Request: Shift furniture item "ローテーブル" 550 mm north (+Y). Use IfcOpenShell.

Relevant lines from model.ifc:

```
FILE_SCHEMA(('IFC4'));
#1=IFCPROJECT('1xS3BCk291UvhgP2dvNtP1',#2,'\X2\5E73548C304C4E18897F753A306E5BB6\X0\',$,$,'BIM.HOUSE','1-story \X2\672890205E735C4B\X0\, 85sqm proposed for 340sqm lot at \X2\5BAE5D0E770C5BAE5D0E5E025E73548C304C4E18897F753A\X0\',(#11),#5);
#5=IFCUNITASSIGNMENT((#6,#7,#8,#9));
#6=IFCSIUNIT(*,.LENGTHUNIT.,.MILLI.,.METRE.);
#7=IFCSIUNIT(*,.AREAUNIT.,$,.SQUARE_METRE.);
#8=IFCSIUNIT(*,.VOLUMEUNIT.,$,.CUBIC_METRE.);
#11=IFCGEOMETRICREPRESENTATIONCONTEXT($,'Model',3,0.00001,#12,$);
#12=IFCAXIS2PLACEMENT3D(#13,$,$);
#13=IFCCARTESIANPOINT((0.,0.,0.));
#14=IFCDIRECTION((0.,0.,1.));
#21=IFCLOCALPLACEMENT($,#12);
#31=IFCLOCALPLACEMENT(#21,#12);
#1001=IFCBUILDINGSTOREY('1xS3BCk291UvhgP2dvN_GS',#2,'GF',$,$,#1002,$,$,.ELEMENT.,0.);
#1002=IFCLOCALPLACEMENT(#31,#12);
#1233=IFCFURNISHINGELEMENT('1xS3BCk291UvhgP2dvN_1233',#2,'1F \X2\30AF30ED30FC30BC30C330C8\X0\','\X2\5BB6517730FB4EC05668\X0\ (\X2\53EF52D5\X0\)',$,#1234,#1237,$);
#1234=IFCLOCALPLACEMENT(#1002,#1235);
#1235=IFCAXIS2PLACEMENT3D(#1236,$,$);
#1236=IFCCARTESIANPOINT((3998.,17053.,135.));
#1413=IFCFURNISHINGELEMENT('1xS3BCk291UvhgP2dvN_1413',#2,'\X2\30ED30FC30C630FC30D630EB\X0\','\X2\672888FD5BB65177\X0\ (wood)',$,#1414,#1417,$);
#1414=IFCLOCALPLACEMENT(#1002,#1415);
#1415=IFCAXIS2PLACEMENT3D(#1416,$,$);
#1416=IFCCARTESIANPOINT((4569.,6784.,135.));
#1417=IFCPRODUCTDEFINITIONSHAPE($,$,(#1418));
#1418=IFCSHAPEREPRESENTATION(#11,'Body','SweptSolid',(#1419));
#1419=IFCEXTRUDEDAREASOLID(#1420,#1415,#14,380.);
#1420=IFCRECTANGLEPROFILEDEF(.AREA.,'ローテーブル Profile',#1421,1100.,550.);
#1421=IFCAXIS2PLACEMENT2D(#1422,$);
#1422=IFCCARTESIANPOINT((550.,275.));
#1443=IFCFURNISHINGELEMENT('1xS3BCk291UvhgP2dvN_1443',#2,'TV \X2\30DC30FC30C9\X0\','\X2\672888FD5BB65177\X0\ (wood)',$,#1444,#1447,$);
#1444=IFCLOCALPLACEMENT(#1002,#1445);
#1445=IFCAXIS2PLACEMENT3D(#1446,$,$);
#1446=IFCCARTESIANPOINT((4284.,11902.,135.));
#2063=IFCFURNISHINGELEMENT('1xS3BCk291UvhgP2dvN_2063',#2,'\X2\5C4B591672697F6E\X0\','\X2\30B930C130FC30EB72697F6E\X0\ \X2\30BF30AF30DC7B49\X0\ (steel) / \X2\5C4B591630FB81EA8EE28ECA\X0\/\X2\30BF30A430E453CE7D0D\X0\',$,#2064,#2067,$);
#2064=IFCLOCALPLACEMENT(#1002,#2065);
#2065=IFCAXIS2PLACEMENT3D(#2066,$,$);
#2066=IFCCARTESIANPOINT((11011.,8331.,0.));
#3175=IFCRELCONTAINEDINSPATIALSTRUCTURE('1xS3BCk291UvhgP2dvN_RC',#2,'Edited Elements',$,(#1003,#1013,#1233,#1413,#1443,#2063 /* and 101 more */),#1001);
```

```python
import ifcopenshell
import ifcopenshell.api.geometry
import ifcopenshell.util.placement

model = ifcopenshell.open("model.ifc")

item = model.by_guid("1xS3BCk291UvhgP2dvN_1413")
matrix = ifcopenshell.util.placement.get_local_placement(item.ObjectPlacement)
matrix[1, 3] += 550.0
ifcopenshell.api.geometry.edit_object_placement(model, product=item, matrix=matrix, is_si=False)

print(ifcopenshell.util.placement.get_local_placement(item.ObjectPlacement).round(3) + 0.0)

model.write("model_updated.ifc")
```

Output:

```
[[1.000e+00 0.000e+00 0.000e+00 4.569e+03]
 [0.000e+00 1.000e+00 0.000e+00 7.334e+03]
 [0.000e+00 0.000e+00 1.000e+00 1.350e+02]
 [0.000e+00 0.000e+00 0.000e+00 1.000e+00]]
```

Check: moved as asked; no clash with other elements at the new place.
